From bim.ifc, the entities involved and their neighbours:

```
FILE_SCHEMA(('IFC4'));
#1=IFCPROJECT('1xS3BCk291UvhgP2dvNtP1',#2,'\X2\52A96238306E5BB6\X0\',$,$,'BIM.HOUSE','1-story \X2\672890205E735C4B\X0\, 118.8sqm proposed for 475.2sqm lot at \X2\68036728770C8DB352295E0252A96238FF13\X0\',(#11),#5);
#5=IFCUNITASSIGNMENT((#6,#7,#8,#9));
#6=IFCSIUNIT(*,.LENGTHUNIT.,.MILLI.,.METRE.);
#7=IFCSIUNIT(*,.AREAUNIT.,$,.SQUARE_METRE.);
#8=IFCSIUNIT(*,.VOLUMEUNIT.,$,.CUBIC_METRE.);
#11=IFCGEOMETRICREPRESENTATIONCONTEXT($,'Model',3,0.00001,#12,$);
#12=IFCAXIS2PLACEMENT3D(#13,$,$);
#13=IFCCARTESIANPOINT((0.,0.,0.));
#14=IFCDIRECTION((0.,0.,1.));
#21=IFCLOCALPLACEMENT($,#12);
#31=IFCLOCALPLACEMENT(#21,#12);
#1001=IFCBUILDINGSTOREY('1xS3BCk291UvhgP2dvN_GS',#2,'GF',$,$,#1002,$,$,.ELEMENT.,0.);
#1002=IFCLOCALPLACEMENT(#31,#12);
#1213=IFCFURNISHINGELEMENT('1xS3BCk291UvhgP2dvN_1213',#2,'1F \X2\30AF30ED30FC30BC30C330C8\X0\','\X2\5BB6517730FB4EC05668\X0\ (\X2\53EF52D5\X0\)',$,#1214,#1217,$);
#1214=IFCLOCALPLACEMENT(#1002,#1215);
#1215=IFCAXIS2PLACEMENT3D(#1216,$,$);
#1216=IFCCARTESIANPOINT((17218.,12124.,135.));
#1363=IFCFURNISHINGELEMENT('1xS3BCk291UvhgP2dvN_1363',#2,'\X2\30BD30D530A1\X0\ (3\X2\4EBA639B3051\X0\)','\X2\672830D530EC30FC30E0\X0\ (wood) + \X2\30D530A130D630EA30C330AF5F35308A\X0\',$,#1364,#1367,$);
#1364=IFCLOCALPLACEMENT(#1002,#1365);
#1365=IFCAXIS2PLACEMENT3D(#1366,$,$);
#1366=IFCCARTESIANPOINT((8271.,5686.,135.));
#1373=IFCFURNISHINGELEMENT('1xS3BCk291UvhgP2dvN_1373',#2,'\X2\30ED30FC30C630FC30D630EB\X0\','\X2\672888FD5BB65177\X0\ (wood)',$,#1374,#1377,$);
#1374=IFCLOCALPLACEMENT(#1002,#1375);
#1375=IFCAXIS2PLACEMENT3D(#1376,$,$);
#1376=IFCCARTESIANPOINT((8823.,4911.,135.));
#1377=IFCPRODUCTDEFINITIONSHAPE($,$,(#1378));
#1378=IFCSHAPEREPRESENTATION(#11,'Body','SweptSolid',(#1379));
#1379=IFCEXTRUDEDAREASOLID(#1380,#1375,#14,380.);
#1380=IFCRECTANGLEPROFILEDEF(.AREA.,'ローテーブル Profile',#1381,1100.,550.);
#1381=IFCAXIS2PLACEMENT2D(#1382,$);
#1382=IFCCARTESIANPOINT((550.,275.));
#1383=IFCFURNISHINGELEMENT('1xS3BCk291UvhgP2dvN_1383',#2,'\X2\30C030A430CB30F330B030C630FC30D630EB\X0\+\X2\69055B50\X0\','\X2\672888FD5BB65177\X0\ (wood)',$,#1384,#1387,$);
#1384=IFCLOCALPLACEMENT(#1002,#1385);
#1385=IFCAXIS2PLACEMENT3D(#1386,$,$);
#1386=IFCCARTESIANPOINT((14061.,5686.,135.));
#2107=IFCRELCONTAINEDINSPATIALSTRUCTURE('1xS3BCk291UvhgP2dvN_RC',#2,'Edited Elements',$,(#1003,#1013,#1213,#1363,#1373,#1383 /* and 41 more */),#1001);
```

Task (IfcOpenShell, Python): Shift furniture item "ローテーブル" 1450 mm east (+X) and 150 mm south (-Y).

```python
import ifcopenshell
import ifcopenshell.api.geometry
import ifcopenshell.util.placement
import ifcopenshell.util.unit

model = ifcopenshell.open("bim.ifc")
unit_scale = ifcopenshell.util.unit.calculate_unit_scale(model)

item = model.by_guid("1xS3BCk291UvhgP2dvN_1373")
matrix = ifcopenshell.util.placement.get_local_placement(item.ObjectPlacement)
matrix[0, 3] += 1.45 / unit_scale
matrix[1, 3] -= 0.15 / unit_scale
ifcopenshell.api.geometry.edit_object_placement(model, product=item, matrix=matrix, is_si=False)

print(ifcopenshell.util.placement.get_local_placement(item.ObjectPlacement).round(3) + 0.0)

model.write("bim_edited.ifc")
```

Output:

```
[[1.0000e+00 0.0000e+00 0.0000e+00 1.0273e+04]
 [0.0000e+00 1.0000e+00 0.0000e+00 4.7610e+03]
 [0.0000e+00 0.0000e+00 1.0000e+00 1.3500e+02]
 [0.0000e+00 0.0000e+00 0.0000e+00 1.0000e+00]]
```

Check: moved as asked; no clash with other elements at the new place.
